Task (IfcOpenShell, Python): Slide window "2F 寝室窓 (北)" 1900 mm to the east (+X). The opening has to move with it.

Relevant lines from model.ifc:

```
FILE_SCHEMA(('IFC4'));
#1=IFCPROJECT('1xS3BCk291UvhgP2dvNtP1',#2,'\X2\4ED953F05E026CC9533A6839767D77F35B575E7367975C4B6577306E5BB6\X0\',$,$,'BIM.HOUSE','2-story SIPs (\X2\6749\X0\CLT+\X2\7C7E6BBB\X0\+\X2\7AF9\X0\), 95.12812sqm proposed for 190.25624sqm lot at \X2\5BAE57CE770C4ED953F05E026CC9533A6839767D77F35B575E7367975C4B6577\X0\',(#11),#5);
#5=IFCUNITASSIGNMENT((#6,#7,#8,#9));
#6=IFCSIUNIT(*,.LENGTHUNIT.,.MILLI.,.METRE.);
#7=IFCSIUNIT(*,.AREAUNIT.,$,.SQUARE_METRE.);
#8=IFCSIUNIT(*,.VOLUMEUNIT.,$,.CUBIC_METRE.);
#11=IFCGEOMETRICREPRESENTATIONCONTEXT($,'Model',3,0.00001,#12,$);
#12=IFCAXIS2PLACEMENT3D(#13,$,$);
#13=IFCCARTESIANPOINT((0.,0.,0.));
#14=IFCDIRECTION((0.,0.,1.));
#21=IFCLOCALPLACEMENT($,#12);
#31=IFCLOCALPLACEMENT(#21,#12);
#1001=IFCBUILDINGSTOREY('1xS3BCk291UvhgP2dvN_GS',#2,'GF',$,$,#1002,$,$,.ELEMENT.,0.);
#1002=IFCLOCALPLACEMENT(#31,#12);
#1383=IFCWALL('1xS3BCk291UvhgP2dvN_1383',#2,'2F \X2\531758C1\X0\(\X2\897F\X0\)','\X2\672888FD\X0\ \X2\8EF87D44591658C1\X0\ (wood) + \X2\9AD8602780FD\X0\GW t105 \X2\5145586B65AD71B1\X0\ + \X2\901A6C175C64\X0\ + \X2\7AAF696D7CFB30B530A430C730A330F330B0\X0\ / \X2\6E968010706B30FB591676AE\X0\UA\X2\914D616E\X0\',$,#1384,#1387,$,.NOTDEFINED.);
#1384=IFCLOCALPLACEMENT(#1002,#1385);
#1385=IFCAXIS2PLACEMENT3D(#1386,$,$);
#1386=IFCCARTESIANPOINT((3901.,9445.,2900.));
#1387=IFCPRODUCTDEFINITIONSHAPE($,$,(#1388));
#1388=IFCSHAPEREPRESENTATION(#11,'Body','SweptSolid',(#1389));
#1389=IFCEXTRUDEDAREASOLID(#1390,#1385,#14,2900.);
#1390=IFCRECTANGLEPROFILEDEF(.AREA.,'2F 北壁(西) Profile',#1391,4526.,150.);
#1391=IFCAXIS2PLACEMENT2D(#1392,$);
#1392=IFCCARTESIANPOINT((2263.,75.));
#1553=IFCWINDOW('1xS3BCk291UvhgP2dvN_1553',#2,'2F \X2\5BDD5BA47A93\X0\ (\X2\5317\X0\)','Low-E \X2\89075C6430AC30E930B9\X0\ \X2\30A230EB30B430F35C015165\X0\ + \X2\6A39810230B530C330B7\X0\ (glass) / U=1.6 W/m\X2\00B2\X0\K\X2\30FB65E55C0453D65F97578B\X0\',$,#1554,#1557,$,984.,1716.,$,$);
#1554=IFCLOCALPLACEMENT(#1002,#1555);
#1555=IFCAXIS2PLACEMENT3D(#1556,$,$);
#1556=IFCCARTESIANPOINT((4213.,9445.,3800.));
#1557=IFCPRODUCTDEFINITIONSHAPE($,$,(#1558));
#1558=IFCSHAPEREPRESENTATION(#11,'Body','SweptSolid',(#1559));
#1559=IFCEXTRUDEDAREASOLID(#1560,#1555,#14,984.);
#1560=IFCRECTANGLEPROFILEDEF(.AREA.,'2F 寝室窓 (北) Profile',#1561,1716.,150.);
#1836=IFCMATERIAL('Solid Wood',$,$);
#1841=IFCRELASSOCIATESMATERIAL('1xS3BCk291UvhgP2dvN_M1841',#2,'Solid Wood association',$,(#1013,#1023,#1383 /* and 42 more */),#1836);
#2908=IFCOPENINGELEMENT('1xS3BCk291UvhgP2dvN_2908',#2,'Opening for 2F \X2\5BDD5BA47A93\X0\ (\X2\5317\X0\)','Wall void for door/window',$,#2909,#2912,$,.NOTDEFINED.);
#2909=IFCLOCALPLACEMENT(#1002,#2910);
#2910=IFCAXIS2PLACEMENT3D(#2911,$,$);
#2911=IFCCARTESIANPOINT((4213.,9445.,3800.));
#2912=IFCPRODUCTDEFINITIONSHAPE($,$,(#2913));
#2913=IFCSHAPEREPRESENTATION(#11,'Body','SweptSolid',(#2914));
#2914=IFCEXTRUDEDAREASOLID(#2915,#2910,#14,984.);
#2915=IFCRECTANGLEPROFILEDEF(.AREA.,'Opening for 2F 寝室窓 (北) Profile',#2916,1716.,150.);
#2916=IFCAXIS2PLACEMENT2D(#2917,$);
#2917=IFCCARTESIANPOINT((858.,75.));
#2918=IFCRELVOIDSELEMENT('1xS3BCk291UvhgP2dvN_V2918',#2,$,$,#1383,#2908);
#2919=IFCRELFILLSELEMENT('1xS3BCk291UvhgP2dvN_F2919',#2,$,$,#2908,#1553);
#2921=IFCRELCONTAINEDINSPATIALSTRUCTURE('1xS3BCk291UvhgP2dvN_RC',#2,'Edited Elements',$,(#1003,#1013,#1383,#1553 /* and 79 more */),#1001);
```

```python
import ifcopenshell
import ifcopenshell.api.geometry
import ifcopenshell.util.placement
import ifcopenshell.util.unit

model = ifcopenshell.open("model.ifc")
unit_scale = ifcopenshell.util.unit.calculate_unit_scale(model)

window = model.by_guid("1xS3BCk291UvhgP2dvN_1553")
opening = window.FillsVoids[0].RelatingOpeningElement
wall = opening.VoidsElements[0].RelatingBuildingElement

wall_matrix = ifcopenshell.util.placement.get_local_placement(wall.ObjectPlacement)
shift = wall_matrix[:3, 0] * 1.9 / unit_scale
before = ifcopenshell.util.placement.get_local_placement(window.ObjectPlacement)[:3, 3].copy()

# The window is not placed relative to its opening, so move both.
for product in (opening, window):
    matrix = ifcopenshell.util.placement.get_local_placement(product.ObjectPlacement)
    matrix[:3, 3] += shift
    ifcopenshell.api.geometry.edit_object_placement(model, product=product, matrix=matrix, is_si=False)

after = ifcopenshell.util.placement.get_local_placement(window.ObjectPlacement)[:3, 3]
print("window moved by", (after - before).round(3) + 0.0)

model.write("model_edited.ifc")
```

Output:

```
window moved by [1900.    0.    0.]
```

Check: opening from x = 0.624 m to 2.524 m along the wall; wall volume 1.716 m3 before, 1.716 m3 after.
